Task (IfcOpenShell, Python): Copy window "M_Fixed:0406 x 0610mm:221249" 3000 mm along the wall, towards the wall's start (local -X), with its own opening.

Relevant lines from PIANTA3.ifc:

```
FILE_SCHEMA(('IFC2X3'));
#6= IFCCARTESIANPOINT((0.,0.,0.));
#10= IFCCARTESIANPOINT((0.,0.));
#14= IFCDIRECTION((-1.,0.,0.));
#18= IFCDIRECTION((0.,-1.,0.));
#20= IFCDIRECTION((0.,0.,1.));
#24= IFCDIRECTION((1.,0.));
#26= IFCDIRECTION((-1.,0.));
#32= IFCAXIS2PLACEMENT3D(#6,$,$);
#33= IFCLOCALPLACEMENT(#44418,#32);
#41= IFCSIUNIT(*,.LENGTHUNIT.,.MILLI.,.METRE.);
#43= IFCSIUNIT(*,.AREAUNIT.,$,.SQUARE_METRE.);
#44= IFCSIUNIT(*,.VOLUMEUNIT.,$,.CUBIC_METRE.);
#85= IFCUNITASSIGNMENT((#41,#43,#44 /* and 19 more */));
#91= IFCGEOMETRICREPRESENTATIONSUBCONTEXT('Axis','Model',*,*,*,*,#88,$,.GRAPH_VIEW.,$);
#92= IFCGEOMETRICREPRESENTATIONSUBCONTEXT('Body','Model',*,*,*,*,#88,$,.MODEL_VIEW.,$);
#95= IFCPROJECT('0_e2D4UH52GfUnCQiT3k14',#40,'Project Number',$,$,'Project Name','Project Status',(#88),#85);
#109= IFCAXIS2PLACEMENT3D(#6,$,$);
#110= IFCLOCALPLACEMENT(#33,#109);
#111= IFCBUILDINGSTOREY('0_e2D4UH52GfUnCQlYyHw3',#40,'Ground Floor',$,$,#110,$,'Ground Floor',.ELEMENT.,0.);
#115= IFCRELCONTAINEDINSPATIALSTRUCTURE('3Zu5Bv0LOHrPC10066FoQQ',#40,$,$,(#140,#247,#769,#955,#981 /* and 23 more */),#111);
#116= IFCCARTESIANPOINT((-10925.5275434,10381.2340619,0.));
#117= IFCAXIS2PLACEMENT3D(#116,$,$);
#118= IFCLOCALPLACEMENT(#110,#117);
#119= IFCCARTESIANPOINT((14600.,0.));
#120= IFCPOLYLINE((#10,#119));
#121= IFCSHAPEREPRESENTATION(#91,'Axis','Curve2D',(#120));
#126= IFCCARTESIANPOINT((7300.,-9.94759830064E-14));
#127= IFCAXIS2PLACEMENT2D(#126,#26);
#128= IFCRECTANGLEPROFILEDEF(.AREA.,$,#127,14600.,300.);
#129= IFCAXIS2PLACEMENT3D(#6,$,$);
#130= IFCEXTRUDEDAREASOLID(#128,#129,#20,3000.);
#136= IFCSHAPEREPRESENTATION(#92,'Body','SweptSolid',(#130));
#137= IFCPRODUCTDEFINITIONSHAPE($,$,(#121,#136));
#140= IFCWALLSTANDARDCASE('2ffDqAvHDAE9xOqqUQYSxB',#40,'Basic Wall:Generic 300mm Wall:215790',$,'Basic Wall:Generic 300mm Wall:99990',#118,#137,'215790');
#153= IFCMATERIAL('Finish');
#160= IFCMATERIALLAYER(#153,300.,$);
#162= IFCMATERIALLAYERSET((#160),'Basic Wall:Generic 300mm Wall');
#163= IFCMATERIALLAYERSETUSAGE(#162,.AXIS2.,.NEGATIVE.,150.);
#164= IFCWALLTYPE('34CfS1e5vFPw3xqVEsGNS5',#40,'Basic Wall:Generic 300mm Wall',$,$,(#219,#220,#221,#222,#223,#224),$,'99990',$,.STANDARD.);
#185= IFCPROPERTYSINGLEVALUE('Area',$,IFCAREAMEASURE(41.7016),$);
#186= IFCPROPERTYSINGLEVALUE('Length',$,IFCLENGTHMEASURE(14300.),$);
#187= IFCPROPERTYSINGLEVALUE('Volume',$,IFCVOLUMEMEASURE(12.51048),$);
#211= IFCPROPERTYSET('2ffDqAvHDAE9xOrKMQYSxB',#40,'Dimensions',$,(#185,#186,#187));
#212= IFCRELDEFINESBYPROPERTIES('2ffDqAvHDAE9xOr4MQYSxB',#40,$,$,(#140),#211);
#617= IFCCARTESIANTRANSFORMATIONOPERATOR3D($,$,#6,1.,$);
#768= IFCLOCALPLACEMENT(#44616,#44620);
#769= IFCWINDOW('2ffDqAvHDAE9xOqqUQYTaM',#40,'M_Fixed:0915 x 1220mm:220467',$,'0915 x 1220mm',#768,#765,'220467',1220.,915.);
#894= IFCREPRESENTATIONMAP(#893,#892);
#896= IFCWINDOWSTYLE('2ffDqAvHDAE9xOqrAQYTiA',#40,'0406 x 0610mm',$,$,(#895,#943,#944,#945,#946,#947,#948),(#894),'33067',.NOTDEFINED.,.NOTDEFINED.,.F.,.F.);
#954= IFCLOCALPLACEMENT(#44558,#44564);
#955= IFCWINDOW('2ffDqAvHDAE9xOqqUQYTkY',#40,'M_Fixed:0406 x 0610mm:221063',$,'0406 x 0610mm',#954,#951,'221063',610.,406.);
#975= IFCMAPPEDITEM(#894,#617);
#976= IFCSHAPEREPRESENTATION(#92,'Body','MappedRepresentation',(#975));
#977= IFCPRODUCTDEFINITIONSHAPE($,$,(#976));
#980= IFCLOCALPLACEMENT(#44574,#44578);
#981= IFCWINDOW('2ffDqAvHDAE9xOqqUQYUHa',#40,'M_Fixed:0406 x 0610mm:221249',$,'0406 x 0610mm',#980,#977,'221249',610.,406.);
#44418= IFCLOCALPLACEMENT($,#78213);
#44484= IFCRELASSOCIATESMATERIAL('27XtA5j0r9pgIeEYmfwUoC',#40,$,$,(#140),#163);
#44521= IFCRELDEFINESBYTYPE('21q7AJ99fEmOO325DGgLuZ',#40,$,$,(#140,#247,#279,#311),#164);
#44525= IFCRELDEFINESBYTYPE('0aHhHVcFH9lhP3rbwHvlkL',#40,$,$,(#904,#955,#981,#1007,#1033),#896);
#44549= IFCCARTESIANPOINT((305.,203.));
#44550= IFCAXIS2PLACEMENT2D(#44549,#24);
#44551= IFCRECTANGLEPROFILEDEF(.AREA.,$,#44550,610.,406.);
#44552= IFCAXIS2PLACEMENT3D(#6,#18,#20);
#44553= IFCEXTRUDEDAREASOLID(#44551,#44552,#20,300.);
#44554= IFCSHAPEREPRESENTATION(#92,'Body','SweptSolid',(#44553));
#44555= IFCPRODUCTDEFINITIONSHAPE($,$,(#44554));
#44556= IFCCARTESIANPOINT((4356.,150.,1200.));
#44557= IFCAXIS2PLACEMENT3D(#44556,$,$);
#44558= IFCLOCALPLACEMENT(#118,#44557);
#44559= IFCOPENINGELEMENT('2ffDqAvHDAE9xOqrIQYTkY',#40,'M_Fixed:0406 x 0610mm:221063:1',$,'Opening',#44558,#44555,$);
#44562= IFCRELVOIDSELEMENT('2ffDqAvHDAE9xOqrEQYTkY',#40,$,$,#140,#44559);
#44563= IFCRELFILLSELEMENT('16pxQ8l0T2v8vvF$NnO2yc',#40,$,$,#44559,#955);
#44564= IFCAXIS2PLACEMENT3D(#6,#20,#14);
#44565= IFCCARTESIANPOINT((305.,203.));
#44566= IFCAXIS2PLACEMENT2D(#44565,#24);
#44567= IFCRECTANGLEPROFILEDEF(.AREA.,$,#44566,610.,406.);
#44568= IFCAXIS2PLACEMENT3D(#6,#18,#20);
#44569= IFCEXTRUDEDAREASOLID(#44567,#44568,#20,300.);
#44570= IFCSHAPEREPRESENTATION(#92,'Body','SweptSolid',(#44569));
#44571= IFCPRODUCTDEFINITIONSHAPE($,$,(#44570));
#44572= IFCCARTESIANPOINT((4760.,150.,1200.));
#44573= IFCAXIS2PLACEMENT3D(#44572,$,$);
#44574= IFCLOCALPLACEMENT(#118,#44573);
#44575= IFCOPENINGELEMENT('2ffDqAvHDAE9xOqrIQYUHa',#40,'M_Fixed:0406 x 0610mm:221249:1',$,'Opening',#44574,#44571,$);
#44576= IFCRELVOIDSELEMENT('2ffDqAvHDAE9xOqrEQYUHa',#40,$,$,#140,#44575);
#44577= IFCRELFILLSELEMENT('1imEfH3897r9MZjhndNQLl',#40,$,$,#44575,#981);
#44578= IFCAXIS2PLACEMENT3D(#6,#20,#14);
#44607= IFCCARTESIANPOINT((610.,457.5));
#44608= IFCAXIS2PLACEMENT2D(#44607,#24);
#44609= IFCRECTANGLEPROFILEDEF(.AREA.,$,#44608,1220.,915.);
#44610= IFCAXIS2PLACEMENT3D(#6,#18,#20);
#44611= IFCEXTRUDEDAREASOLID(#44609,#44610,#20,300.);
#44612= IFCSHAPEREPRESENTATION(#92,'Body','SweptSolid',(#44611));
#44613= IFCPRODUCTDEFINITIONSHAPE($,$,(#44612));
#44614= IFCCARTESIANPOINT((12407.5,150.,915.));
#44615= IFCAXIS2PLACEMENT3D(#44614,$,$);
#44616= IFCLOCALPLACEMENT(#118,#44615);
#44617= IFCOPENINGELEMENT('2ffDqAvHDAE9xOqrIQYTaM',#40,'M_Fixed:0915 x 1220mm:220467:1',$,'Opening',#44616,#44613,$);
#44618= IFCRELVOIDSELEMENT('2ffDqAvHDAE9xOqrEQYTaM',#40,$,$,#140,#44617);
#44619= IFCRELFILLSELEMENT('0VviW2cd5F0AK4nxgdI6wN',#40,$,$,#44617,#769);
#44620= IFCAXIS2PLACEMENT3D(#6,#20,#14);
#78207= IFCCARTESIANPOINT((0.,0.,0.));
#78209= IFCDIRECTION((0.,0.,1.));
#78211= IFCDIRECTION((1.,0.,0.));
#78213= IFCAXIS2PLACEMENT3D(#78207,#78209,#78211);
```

```python
import ifcopenshell
import ifcopenshell.api.feature
import ifcopenshell.api.geometry
import ifcopenshell.api.pset
import ifcopenshell.api.root
import ifcopenshell.geom
import ifcopenshell.util.element
import ifcopenshell.util.placement
import ifcopenshell.util.shape
import ifcopenshell.util.unit

model = ifcopenshell.open("PIANTA3.ifc")
unit_scale = ifcopenshell.util.unit.calculate_unit_scale(model)
area_scale = ifcopenshell.util.unit.calculate_unit_scale(model, "AREAUNIT")
volume_scale = ifcopenshell.util.unit.calculate_unit_scale(model, "VOLUMEUNIT")
settings = ifcopenshell.geom.settings()


def volume(element):
    """Net volume in cubic metres, openings subtracted."""
    shape = ifcopenshell.geom.create_shape(settings, element)
    return ifcopenshell.util.shape.get_volume(shape.geometry)


def reuse_history(source, copy):
    """copy_class also copies each property set's owner history, people and application; keep the originals."""
    for rel in copy.IsDefinedBy:
        if rel.is_a("IfcRelDefinesByProperties") and (history := rel.RelatingPropertyDefinition.OwnerHistory):
            rel.RelatingPropertyDefinition.OwnerHistory = source.OwnerHistory
            ifcopenshell.util.element.remove_deep2(model, history)


window = model.by_id(981)
opening = window.FillsVoids[0].RelatingOpeningElement
wall = opening.VoidsElements[0].RelatingBuildingElement
before = volume(wall)
shift = ifcopenshell.util.placement.get_local_placement(wall.ObjectPlacement)[:3, 0] * -3 / unit_scale

# copy_class copies the void relationship, type, container and properties, but no geometry.
new_opening = ifcopenshell.api.root.copy_class(model, product=opening)
new_opening.Representation = ifcopenshell.util.element.copy_deep(
    model, opening.Representation, exclude=["IfcGeometricRepresentationContext", "IfcRepresentationMap"]
)
new_opening.Name = "M_Fixed:0406 x 0610mm"
new_window = ifcopenshell.api.root.copy_class(model, product=window)
new_window.Representation = ifcopenshell.util.element.copy_deep(
    model, window.Representation, exclude=["IfcGeometricRepresentationContext", "IfcRepresentationMap"]
)
new_window.Name = "M_Fixed:0406 x 0610mm"
new_window.Tag = None
reuse_history(window, new_window)
fills = ifcopenshell.api.feature.add_filling(model, opening=new_opening, element=new_window)
fills.OwnerHistory = new_window.OwnerHistory  # required in IFC2X3

for old, new in ((opening, new_opening), (window, new_window)):
    matrix = ifcopenshell.util.placement.get_local_placement(old.ObjectPlacement)
    matrix[:3, 3] += shift
    ifcopenshell.api.geometry.edit_object_placement(model, product=new, matrix=matrix, is_si=False)

after = volume(wall)
thickness = 0.3  # wall thickness in metres

# Update the wall's stored quantities.
pset = model.by_id(ifcopenshell.util.element.get_pset(wall, "Dimensions", should_inherit=False)["id"])
ifcopenshell.api.pset.edit_pset(model, pset=pset, properties={
    "Area": model.create_entity("IfcAreaMeasure", after / thickness / area_scale),
    "Volume": model.create_entity("IfcVolumeMeasure", after / volume_scale),
})

print(f"wall volume {before:.3f} -> {after:.3f} m3")

model.write("PIANTA3_edited.ifc")
```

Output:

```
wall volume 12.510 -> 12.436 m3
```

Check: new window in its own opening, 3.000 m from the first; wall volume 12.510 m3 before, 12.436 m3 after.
